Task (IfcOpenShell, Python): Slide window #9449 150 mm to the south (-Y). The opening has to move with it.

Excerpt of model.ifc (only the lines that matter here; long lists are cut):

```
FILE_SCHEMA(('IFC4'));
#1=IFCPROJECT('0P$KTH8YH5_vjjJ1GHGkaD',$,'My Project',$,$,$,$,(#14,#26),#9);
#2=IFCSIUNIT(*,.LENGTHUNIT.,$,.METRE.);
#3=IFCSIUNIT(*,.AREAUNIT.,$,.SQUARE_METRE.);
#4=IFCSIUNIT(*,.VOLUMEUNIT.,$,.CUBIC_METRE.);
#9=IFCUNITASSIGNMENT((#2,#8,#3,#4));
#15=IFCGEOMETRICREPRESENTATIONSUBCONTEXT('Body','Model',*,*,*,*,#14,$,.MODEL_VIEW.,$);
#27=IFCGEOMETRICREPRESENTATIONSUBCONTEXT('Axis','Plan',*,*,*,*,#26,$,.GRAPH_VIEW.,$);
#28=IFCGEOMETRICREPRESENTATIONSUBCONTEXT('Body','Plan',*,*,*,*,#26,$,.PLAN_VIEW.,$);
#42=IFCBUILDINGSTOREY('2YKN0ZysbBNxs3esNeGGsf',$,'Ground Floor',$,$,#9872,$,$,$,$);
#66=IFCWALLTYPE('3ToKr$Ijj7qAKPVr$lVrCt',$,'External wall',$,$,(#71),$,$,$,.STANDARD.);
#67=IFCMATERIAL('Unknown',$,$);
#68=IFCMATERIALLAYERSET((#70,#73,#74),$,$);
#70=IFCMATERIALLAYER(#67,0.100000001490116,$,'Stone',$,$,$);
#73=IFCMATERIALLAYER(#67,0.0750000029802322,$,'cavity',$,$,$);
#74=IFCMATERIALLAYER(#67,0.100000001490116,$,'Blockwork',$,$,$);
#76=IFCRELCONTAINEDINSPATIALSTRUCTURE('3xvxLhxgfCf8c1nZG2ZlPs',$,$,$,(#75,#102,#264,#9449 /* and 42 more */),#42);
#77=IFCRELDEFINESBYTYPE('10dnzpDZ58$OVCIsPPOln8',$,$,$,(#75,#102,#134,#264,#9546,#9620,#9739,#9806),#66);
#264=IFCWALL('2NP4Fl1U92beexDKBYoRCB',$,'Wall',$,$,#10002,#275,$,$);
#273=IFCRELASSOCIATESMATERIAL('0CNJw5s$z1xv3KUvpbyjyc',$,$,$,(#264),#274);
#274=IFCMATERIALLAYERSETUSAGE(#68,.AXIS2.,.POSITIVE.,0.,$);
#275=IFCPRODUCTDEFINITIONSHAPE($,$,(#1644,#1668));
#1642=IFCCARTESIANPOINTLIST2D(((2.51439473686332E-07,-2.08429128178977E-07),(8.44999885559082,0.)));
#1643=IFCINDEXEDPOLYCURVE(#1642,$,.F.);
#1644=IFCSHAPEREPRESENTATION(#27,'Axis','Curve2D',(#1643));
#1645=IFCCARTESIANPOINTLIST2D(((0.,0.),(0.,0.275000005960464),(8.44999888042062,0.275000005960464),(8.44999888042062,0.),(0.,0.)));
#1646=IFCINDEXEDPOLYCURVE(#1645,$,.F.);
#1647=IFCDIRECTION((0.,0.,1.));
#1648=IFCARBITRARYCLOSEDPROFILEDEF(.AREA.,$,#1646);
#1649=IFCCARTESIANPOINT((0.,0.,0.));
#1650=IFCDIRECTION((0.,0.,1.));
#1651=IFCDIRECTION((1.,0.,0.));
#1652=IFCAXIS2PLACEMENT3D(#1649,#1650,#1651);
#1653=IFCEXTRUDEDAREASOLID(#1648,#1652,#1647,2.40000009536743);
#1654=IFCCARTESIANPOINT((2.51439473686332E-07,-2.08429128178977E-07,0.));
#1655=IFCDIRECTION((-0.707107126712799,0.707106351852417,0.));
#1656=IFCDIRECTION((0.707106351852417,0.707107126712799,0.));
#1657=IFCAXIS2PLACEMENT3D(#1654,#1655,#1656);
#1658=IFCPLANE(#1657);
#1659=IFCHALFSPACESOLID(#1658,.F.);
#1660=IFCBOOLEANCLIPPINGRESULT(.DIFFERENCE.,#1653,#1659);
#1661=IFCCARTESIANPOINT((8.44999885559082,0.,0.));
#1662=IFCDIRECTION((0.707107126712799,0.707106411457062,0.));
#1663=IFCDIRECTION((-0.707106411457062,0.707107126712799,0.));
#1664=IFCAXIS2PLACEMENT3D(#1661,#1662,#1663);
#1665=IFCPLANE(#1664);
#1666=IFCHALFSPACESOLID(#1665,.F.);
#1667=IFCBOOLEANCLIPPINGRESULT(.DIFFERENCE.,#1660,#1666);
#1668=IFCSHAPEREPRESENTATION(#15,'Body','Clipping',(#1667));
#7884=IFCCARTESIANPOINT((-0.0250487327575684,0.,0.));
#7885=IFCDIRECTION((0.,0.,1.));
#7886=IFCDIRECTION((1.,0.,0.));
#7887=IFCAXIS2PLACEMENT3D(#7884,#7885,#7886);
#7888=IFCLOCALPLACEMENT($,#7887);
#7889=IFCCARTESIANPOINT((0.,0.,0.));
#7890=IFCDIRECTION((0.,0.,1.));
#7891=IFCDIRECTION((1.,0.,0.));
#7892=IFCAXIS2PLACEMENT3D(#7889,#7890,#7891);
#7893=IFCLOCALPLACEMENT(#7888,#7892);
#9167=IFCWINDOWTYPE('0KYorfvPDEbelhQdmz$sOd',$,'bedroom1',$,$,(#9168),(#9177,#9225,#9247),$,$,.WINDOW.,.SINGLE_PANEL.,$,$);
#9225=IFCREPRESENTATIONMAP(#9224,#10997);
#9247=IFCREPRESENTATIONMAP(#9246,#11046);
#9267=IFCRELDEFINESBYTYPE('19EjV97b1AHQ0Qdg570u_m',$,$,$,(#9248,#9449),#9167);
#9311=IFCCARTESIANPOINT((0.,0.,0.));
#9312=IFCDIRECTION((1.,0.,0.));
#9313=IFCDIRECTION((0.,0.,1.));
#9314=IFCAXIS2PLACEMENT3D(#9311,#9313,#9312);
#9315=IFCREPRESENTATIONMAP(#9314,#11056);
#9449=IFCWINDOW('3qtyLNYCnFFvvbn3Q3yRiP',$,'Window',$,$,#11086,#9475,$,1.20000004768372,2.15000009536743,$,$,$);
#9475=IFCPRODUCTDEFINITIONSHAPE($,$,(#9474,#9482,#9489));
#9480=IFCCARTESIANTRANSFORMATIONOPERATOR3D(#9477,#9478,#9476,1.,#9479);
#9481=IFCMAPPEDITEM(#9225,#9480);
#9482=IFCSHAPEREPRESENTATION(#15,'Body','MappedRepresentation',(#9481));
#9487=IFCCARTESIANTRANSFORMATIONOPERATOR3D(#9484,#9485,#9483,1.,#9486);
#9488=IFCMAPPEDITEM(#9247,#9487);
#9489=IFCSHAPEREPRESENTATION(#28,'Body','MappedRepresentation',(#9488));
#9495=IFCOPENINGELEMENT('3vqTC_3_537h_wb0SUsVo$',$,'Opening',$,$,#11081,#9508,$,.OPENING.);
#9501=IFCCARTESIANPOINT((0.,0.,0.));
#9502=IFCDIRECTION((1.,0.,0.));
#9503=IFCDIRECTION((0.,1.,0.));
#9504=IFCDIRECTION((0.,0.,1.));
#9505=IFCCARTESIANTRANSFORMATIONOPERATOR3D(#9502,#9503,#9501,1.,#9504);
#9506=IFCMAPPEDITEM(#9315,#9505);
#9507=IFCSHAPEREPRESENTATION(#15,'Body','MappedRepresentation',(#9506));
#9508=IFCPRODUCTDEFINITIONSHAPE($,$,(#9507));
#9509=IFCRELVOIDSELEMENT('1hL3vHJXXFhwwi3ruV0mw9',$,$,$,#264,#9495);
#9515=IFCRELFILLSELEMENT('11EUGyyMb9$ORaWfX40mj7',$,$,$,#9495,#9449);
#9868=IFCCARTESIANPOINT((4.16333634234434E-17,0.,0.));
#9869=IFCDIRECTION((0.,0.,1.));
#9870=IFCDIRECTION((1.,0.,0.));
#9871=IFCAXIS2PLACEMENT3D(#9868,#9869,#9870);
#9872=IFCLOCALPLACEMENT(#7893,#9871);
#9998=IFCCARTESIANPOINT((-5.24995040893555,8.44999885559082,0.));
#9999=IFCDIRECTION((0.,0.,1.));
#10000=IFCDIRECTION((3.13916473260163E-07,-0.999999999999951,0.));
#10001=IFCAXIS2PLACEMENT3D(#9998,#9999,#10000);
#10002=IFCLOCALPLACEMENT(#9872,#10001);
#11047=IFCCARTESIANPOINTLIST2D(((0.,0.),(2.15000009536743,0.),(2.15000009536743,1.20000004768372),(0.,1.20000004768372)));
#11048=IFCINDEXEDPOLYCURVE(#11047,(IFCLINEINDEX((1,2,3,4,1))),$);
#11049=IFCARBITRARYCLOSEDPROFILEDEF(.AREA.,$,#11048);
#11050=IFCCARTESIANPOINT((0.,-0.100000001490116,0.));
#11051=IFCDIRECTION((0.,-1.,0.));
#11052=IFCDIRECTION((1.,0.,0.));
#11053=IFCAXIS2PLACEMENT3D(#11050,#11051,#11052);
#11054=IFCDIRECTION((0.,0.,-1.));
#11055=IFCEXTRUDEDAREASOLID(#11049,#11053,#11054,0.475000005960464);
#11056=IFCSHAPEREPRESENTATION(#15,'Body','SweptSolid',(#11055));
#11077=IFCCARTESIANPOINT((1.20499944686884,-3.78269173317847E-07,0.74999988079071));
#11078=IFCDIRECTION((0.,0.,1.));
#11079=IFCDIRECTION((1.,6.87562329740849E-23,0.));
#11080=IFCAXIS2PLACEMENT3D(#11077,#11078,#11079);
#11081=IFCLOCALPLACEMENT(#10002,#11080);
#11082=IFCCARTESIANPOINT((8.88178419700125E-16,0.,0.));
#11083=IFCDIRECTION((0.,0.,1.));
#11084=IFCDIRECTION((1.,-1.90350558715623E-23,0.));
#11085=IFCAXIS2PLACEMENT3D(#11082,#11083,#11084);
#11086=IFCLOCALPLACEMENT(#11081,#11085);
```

```python
import ifcopenshell
import ifcopenshell.api.geometry
import ifcopenshell.util.placement

model = ifcopenshell.open("model.ifc")

window = model.by_guid("3qtyLNYCnFFvvbn3Q3yRiP")
opening = window.FillsVoids[0].RelatingOpeningElement
wall = opening.VoidsElements[0].RelatingBuildingElement

wall_matrix = ifcopenshell.util.placement.get_local_placement(wall.ObjectPlacement)
shift = wall_matrix[:3, 0] * 0.15
before = ifcopenshell.util.placement.get_local_placement(window.ObjectPlacement)[:3, 3].copy()

# The window is placed relative to its opening, so it follows when the opening moves.
matrix = ifcopenshell.util.placement.get_local_placement(opening.ObjectPlacement)
matrix[:3, 3] += shift
ifcopenshell.api.geometry.edit_object_placement(
    model, product=opening, matrix=matrix, is_si=False, should_transform_children=True
)

after = ifcopenshell.util.placement.get_local_placement(window.ObjectPlacement)[:3, 3]
print("window moved by", (after - before).round(3) + 0.0)

model.write("model_v2.ifc")
```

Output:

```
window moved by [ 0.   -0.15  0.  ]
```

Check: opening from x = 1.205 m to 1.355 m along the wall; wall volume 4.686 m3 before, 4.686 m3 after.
